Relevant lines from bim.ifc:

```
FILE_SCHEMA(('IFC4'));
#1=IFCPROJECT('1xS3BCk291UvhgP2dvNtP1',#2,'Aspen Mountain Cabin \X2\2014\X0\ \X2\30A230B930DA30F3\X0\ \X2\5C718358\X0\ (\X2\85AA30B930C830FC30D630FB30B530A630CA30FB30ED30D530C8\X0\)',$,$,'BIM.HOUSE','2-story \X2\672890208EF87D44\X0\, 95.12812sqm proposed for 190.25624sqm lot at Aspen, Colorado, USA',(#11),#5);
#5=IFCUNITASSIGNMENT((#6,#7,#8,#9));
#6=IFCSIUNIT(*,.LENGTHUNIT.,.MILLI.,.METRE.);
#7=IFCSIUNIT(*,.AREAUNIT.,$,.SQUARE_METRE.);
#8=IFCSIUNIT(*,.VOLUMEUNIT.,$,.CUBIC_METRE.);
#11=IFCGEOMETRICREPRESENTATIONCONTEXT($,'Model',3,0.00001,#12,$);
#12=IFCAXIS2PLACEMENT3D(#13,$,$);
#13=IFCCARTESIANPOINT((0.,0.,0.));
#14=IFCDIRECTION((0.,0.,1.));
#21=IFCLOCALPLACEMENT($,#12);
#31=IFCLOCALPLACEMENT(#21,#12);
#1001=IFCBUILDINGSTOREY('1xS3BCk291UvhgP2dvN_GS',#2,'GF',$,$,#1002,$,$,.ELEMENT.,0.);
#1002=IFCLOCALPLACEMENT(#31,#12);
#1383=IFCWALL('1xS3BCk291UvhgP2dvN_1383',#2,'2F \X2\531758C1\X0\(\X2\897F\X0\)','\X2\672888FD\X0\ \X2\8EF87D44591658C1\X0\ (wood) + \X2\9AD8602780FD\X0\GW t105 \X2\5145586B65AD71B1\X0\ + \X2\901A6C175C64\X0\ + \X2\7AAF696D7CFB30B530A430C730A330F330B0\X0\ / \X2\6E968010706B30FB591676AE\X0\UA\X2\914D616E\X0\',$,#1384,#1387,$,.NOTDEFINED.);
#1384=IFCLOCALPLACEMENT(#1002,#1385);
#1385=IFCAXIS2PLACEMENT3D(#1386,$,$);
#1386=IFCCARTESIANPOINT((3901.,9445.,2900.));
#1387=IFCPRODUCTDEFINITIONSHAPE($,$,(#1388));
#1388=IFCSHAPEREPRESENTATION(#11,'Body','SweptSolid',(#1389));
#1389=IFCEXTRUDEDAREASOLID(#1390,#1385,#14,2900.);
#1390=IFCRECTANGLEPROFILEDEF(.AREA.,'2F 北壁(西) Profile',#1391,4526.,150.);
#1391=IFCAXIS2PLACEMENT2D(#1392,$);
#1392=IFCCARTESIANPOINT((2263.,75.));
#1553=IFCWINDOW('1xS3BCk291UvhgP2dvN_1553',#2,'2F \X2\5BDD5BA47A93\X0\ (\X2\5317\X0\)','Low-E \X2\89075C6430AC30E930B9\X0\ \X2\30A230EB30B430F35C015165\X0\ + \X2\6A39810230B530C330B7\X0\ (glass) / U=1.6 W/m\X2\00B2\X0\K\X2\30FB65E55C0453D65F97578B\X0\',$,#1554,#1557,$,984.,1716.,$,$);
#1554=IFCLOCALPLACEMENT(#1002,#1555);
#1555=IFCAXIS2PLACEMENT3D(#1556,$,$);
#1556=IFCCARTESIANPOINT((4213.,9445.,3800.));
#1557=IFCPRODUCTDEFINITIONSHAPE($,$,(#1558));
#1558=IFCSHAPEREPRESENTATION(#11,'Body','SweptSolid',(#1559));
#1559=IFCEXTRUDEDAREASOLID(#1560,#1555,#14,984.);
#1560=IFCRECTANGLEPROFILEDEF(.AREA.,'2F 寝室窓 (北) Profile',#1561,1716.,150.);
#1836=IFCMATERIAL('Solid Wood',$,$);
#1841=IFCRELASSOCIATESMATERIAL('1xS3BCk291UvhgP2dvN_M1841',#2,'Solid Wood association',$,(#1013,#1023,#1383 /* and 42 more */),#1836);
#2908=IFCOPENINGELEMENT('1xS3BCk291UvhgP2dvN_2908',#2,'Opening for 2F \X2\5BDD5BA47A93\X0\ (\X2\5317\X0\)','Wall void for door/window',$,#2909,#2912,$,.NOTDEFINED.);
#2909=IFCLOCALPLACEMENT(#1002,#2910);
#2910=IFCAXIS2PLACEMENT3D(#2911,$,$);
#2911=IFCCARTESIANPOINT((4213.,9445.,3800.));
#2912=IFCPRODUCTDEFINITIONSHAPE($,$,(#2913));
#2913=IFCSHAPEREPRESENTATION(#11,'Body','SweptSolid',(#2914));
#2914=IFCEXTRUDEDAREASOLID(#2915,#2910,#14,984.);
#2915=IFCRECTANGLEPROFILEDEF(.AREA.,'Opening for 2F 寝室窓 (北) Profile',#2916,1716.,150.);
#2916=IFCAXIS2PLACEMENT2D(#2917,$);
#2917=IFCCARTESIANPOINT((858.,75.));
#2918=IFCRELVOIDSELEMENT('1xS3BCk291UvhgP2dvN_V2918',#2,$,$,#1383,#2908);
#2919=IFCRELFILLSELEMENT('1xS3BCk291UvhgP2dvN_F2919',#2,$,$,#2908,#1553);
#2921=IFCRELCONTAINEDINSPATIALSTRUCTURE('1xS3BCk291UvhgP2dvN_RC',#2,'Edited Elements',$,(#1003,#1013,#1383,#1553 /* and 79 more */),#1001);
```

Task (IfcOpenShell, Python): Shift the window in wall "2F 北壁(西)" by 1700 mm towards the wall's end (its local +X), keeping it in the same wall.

```python
import ifcopenshell
import ifcopenshell.api.geometry
import ifcopenshell.util.placement

model = ifcopenshell.open("bim.ifc")

window = model.by_guid("1xS3BCk291UvhgP2dvN_1553")
opening = window.FillsVoids[0].RelatingOpeningElement
wall = opening.VoidsElements[0].RelatingBuildingElement

wall_matrix = ifcopenshell.util.placement.get_local_placement(wall.ObjectPlacement)
shift = wall_matrix[:3, 0] * 1700.0
before = ifcopenshell.util.placement.get_local_placement(window.ObjectPlacement)[:3, 3].copy()

# The window is not placed relative to its opening, so move both.
for product in (opening, window):
    matrix = ifcopenshell.util.placement.get_local_placement(product.ObjectPlacement)
    matrix[:3, 3] += shift
    ifcopenshell.api.geometry.edit_object_placement(model, product=product, matrix=matrix, is_si=False)

after = ifcopenshell.util.placement.get_local_placement(window.ObjectPlacement)[:3, 3]
print("window moved by", (after - before).round(3) + 0.0)

model.write("bim_edited.ifc")
```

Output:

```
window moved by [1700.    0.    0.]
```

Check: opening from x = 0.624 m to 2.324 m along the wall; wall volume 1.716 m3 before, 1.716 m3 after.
